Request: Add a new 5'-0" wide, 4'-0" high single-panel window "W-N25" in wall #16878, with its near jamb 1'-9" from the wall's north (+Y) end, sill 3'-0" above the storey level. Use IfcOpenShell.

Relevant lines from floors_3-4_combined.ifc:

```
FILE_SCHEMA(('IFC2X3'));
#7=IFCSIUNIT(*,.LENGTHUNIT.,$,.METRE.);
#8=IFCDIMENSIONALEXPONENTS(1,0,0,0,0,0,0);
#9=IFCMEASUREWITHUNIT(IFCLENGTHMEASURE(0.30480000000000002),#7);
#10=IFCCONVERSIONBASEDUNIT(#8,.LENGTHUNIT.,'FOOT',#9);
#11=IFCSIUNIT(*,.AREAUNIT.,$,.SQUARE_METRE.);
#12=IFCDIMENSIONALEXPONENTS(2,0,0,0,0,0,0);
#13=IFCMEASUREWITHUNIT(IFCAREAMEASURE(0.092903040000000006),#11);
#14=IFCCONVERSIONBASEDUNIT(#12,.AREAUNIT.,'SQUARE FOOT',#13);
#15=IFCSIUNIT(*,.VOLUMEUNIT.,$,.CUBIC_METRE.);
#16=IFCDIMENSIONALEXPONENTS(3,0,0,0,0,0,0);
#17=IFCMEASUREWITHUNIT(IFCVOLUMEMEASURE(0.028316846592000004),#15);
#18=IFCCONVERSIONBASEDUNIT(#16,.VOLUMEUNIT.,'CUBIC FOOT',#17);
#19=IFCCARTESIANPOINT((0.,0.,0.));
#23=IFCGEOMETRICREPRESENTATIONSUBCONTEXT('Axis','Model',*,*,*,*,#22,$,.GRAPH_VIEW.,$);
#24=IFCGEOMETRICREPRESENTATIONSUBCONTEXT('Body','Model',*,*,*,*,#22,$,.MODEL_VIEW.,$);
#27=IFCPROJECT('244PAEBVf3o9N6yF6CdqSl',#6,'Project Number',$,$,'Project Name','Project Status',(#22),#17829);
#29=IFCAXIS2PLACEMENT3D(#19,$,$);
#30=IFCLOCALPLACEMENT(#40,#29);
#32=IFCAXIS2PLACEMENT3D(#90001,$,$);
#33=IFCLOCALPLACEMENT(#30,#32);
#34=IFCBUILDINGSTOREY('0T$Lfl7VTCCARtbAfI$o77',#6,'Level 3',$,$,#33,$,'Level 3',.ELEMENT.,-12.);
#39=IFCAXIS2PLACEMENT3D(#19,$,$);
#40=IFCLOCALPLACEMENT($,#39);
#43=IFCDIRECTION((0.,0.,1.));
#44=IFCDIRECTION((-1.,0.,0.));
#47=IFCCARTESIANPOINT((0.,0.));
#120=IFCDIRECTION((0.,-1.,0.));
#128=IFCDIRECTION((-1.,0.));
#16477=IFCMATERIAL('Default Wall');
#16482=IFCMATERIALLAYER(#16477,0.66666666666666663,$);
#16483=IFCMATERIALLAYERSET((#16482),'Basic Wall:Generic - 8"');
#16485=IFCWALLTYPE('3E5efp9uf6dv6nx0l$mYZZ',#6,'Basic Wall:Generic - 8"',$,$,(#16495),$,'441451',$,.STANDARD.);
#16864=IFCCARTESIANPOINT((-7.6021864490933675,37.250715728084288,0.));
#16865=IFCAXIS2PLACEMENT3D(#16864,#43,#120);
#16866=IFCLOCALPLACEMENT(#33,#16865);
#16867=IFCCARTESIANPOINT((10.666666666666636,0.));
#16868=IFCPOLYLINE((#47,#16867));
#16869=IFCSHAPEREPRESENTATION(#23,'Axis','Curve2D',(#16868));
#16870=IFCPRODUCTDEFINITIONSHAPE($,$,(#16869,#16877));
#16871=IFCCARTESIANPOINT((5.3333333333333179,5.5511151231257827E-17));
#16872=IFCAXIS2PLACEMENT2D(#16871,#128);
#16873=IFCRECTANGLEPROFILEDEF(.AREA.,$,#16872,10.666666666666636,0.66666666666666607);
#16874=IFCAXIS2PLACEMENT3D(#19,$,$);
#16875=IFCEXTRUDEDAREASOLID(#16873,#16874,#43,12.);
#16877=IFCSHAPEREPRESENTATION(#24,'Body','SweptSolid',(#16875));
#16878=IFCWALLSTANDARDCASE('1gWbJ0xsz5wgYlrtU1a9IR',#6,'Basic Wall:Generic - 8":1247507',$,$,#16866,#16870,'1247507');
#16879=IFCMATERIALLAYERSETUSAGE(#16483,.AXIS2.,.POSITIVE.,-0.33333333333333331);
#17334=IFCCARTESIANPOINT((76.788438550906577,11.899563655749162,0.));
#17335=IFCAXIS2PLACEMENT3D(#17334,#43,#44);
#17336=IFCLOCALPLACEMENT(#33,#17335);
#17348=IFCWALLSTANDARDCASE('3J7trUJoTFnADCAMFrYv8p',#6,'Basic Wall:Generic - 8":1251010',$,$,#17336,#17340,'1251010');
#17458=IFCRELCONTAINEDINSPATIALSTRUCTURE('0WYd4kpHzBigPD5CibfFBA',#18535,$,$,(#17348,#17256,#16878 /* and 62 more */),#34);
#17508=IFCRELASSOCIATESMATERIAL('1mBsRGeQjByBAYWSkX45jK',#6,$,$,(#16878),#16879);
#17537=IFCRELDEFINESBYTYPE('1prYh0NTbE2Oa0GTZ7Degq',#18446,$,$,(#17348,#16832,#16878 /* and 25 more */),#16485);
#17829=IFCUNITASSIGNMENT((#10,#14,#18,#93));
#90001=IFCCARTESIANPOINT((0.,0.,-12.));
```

```python
import numpy as np
import ifcopenshell
import ifcopenshell.api.feature
import ifcopenshell.api.geometry
import ifcopenshell.api.root
import ifcopenshell.api.spatial
import ifcopenshell.api.type
import ifcopenshell.geom
import ifcopenshell.util.element
import ifcopenshell.util.placement
import ifcopenshell.util.representation
import ifcopenshell.util.shape
import ifcopenshell.util.unit

model = ifcopenshell.open("floors_3-4_combined.ifc")
unit_scale = ifcopenshell.util.unit.calculate_unit_scale(model)
settings = ifcopenshell.geom.settings()


def volume(element):
    """Net volume in cubic metres, openings subtracted."""
    shape = ifcopenshell.geom.create_shape(settings, element)
    return ifcopenshell.util.shape.get_volume(shape.geometry)


wall = model.by_id(16878)
storey = ifcopenshell.util.element.get_container(wall, ifc_class="IfcBuildingStorey")
context = ifcopenshell.util.representation.get_context(model, "Model", "Body", "MODEL_VIEW")
before = volume(wall)

width, height, from_end, sill = 1.524, 1.2192, 0.5334, 0.9144  # metres

# The wall runs along its own X axis, and the end named is its -X end.
wall_shape = ifcopenshell.geom.create_shape(settings, wall)
x, y, z = ifcopenshell.util.shape.get_vertices(wall_shape.geometry).T
start = x.min() + from_end
face, thickness = float(y.min()), float(y.max() - y.min())
wall_matrix = ifcopenshell.util.placement.get_local_placement(wall.ObjectPlacement)
level = ifcopenshell.util.placement.get_local_placement(storey.ObjectPlacement)[2, 3]


def in_wall(x, y):
    """Placement at x, y metres in the wall's axes, at sill height."""
    matrix = wall_matrix.copy()
    matrix[:, 3] = wall_matrix @ np.array([x / unit_scale, y / unit_scale, 0.0, 1.0])
    matrix[2, 3] = level + sill / unit_scale
    return matrix


# Opening: a box that overshoots both wall faces by 50 mm.
opening = ifcopenshell.api.root.create_entity(model, ifc_class="IfcOpeningElement")
box = ifcopenshell.api.geometry.add_wall_representation(
    model, context=context, length=width, height=height, thickness=thickness + 0.1
)
ifcopenshell.api.geometry.assign_representation(model, product=opening, representation=box)
ifcopenshell.api.geometry.edit_object_placement(model, product=opening, matrix=in_wall(start, face - 0.05), is_si=False)
ifcopenshell.api.feature.add_feature(model, feature=opening, element=wall)

window = ifcopenshell.api.root.create_entity(model, ifc_class="IfcWindow", name="W-N25")
window.OverallWidth, window.OverallHeight = width / unit_scale, height / unit_scale
body = ifcopenshell.api.geometry.add_window_representation(
    model,
    context=context,
    overall_width=window.OverallWidth,
    overall_height=window.OverallHeight,
    partition_type="SINGLE_PANEL",
)
ifcopenshell.api.geometry.assign_representation(model, product=window, representation=body)
ifcopenshell.api.spatial.assign_container(model, products=[window], relating_structure=storey)
fills = ifcopenshell.api.feature.add_filling(model, opening=opening, element=window)
fills.OwnerHistory = window.OwnerHistory  # required in IFC2X3

# IFC2X3 keeps the operation on the window style.
style = ifcopenshell.api.root.create_entity(model, ifc_class="IfcWindowStyle", name="W-N25")
style.OperationType, style.ConstructionType = "SINGLE_PANEL", "NOTDEFINED"
style.ParameterTakesPrecedence = style.Sizeable = False
ifcopenshell.api.type.assign_type(model, related_objects=[window], relating_type=style)

# Centre the window in the wall's thickness.
ifcopenshell.api.geometry.edit_object_placement(model, product=window, matrix=in_wall(start, face), is_si=False)
window_shape = ifcopenshell.geom.create_shape(settings, window)
depth = ifcopenshell.util.shape.get_vertices(window_shape.geometry)[:, 1]
offset = face + thickness / 2 - (depth.min() + depth.max()) / 2
ifcopenshell.api.geometry.edit_object_placement(model, product=window, matrix=in_wall(start, offset), is_si=False)

after = volume(wall)

print(f"wall volume {before:.3f} -> {after:.3f} m3")

model.write("floors_3-4_combined_updated.ifc")
```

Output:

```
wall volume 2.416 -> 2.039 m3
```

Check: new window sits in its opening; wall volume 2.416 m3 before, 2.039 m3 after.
